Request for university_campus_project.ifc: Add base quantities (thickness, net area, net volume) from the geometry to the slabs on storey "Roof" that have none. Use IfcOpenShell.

First a look at what the model holds.

```python
import ifcopenshell
import ifcopenshell.util.element
import ifcopenshell.util.unit

model = ifcopenshell.open("university_campus_project.ifc")
print(model.schema)
for unit_type in ("LENGTHUNIT", "AREAUNIT", "VOLUMEUNIT"):
    print(unit_type, ifcopenshell.util.unit.calculate_unit_scale(model, unit_type))
storey = next(s for s in model.by_type("IfcBuildingStorey") if s.Name == "Roof")
slabs = [e for e in ifcopenshell.util.element.get_decomposition(storey) if e.is_a("IfcSlab")]
for e in sorted(slabs, key=lambda e: e.id()):
    print(e.id(), e.is_a(), e.Name, list(ifcopenshell.util.element.get_psets(e, qtos_only=True)), sep=" | ")
```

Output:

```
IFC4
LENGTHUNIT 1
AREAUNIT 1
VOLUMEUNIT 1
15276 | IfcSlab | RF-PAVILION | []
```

```python
import ifcopenshell
import ifcopenshell.api.pset
import ifcopenshell.geom
import ifcopenshell.util.element
import ifcopenshell.util.shape
import ifcopenshell.util.unit

model = ifcopenshell.open("university_campus_project.ifc")
unit_scale = ifcopenshell.util.unit.calculate_unit_scale(model)
area_scale = ifcopenshell.util.unit.calculate_unit_scale(model, "AREAUNIT")
volume_scale = ifcopenshell.util.unit.calculate_unit_scale(model, "VOLUMEUNIT")
settings = ifcopenshell.geom.settings()

storey = next(s for s in model.by_type("IfcBuildingStorey") if s.Name == "Roof")
slabs = [e for e in ifcopenshell.util.element.get_decomposition(storey) if e.is_a("IfcSlab")]

for e in sorted(slabs, key=lambda e: e.id()):
    if ifcopenshell.util.element.get_psets(e, qtos_only=True, should_inherit=False):
        continue
    # Geometry comes back in metres, in the element's own axes.
    shape = ifcopenshell.geom.create_shape(settings, e)
    values = {
        "Width": ifcopenshell.util.shape.get_z(shape.geometry) / unit_scale,
        "NetArea": ifcopenshell.util.shape.get_footprint_area(shape.geometry) / area_scale,
        "NetVolume": ifcopenshell.util.shape.get_volume(shape.geometry) / volume_scale,
    }
    qto = ifcopenshell.api.pset.add_qto(model, product=e, name="Qto_SlabBaseQuantities")
    ifcopenshell.api.pset.edit_qto(model, qto=qto, properties=values)
    print(e.id(), {k: round(v, 3) for k, v in values.items()})

model.write("university_campus_project_updated.ifc")
```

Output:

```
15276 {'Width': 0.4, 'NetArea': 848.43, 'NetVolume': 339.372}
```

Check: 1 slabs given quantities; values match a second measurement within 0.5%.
